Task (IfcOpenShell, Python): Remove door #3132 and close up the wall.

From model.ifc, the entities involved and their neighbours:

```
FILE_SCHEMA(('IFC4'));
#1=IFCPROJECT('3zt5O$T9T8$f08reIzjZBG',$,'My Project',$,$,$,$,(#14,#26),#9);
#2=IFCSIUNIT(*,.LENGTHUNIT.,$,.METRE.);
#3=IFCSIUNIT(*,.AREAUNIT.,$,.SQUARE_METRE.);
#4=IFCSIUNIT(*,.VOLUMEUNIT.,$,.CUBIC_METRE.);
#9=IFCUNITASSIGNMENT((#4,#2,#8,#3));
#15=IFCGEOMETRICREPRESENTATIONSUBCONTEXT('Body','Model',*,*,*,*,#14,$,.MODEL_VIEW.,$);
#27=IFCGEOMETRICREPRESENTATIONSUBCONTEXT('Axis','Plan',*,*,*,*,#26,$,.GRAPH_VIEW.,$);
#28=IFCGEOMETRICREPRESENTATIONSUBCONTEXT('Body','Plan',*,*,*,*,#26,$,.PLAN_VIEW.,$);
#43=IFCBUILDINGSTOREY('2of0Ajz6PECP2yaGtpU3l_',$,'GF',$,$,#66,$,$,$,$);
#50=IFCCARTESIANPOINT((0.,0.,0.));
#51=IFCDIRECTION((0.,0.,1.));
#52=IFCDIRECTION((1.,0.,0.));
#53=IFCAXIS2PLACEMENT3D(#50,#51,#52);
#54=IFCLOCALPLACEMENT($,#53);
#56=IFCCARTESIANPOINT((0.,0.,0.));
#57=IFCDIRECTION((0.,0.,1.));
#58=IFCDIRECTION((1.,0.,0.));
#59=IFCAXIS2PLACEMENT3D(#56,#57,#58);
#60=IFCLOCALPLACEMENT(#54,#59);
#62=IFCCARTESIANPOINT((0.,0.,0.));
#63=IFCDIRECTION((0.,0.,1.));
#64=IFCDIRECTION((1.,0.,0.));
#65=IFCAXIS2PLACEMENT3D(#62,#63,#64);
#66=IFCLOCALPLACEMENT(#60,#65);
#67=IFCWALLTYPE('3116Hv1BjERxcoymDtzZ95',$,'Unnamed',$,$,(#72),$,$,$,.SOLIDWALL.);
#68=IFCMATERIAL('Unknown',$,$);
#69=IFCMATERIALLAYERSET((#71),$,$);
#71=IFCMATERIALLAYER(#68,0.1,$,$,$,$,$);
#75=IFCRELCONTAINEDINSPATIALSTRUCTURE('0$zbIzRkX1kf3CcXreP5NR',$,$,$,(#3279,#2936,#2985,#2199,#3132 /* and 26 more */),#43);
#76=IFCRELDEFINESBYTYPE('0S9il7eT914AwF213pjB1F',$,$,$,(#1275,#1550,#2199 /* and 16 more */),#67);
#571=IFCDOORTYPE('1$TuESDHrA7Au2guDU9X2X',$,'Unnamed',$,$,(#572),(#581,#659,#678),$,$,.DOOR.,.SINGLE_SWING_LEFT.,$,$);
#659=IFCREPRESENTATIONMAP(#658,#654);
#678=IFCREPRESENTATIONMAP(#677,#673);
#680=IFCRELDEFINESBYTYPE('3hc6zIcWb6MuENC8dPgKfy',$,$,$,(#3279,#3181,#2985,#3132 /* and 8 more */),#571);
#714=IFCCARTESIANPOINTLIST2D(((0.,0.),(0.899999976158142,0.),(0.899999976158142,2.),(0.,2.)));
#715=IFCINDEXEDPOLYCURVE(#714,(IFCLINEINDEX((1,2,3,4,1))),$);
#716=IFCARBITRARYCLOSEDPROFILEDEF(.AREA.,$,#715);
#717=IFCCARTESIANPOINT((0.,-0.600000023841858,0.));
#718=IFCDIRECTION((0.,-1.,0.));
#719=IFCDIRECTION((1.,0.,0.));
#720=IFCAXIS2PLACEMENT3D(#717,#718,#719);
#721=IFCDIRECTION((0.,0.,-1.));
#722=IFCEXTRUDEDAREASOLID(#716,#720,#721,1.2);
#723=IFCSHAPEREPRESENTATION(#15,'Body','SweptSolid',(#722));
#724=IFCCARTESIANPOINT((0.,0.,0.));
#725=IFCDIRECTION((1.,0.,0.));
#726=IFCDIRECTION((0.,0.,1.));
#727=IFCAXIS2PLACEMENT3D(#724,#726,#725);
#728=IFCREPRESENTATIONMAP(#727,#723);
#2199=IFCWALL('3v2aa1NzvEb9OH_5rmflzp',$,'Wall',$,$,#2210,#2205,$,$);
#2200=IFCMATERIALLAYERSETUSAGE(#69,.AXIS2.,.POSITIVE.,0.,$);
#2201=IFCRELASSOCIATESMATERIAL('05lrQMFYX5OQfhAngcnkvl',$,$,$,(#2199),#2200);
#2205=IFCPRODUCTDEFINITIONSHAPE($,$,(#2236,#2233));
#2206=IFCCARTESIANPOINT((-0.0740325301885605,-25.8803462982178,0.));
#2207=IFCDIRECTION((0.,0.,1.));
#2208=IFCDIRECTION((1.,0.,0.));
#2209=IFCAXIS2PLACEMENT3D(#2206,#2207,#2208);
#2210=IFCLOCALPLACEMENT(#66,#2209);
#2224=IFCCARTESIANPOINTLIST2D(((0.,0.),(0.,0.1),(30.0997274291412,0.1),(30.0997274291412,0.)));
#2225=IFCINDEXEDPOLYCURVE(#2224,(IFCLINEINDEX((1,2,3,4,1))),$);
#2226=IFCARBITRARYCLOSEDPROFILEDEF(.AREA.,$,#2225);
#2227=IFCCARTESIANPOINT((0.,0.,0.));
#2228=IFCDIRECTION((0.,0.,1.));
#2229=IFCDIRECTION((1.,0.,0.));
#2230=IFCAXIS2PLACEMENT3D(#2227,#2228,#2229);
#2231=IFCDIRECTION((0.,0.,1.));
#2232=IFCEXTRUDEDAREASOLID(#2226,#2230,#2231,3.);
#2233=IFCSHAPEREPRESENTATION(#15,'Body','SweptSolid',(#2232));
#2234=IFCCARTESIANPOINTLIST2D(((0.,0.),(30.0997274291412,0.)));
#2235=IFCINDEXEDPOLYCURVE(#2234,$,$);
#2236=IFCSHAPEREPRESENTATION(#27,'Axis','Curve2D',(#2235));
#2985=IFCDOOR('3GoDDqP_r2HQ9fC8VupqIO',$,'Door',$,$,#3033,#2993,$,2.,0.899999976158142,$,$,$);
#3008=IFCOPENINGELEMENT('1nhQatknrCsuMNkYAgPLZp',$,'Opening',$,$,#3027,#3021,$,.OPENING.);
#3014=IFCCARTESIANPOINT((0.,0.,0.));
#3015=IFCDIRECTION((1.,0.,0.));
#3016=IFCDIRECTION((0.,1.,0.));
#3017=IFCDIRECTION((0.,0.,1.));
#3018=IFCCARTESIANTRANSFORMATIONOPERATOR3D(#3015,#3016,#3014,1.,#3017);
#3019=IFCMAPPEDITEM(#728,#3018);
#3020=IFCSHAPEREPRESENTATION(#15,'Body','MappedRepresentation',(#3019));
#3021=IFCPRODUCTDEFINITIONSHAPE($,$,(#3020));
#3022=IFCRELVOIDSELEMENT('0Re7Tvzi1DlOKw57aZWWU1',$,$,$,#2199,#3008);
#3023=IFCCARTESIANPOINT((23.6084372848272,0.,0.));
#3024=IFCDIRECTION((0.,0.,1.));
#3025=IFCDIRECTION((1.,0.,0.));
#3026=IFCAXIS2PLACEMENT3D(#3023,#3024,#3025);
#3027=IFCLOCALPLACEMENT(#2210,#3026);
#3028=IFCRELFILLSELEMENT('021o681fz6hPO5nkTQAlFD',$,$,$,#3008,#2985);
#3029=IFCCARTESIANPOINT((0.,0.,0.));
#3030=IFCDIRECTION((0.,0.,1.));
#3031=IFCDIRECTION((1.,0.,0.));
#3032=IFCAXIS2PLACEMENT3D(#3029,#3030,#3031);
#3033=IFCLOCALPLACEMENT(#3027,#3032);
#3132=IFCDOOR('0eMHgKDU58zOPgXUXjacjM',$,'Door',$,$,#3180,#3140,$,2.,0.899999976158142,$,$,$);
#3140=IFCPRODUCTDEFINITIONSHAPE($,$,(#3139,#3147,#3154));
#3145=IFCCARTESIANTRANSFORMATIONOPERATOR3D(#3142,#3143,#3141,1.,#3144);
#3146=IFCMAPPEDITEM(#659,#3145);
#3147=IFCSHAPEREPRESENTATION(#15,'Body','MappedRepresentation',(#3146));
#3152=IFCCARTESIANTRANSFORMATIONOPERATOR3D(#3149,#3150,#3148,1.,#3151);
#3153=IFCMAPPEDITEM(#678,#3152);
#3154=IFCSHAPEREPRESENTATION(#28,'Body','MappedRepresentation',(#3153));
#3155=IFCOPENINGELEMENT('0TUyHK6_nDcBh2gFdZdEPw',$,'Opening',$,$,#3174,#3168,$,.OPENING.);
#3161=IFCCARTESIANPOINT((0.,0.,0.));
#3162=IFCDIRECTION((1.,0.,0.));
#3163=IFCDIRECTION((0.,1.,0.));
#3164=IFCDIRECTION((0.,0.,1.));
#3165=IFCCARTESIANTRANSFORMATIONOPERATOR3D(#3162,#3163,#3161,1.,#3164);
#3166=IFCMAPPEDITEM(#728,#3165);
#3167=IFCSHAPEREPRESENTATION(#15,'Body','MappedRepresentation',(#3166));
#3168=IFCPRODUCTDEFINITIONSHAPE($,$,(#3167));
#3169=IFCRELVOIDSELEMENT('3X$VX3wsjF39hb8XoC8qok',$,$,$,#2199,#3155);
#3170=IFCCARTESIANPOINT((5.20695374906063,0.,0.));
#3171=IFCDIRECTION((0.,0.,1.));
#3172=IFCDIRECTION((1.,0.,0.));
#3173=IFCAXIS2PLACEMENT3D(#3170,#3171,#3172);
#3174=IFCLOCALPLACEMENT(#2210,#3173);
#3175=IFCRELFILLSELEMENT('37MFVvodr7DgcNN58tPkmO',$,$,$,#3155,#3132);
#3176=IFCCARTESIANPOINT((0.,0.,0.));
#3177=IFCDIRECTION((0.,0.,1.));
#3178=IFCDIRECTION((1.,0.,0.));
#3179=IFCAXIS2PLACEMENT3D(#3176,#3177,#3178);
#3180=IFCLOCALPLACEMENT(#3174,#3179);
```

```python
import ifcopenshell
import ifcopenshell.api.feature
import ifcopenshell.api.root
import ifcopenshell.geom
import ifcopenshell.util.shape

model = ifcopenshell.open("model.ifc")
settings = ifcopenshell.geom.settings()


def volume(element):
    """Net volume in cubic metres, openings subtracted."""
    shape = ifcopenshell.geom.create_shape(settings, element)
    return ifcopenshell.util.shape.get_volume(shape.geometry)


door = model.by_guid("0eMHgKDU58zOPgXUXjacjM")
opening = door.FillsVoids[0].RelatingOpeningElement
wall = opening.VoidsElements[0].RelatingBuildingElement
before = volume(wall)

ifcopenshell.api.root.remove_product(model, product=door)
ifcopenshell.api.feature.remove_feature(model, feature=opening)

after = volume(wall)

print(f"wall volume {before:.3f} -> {after:.3f} m3")

model.write("model_edited.ifc")
```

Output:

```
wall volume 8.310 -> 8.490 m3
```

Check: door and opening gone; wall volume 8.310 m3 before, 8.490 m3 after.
